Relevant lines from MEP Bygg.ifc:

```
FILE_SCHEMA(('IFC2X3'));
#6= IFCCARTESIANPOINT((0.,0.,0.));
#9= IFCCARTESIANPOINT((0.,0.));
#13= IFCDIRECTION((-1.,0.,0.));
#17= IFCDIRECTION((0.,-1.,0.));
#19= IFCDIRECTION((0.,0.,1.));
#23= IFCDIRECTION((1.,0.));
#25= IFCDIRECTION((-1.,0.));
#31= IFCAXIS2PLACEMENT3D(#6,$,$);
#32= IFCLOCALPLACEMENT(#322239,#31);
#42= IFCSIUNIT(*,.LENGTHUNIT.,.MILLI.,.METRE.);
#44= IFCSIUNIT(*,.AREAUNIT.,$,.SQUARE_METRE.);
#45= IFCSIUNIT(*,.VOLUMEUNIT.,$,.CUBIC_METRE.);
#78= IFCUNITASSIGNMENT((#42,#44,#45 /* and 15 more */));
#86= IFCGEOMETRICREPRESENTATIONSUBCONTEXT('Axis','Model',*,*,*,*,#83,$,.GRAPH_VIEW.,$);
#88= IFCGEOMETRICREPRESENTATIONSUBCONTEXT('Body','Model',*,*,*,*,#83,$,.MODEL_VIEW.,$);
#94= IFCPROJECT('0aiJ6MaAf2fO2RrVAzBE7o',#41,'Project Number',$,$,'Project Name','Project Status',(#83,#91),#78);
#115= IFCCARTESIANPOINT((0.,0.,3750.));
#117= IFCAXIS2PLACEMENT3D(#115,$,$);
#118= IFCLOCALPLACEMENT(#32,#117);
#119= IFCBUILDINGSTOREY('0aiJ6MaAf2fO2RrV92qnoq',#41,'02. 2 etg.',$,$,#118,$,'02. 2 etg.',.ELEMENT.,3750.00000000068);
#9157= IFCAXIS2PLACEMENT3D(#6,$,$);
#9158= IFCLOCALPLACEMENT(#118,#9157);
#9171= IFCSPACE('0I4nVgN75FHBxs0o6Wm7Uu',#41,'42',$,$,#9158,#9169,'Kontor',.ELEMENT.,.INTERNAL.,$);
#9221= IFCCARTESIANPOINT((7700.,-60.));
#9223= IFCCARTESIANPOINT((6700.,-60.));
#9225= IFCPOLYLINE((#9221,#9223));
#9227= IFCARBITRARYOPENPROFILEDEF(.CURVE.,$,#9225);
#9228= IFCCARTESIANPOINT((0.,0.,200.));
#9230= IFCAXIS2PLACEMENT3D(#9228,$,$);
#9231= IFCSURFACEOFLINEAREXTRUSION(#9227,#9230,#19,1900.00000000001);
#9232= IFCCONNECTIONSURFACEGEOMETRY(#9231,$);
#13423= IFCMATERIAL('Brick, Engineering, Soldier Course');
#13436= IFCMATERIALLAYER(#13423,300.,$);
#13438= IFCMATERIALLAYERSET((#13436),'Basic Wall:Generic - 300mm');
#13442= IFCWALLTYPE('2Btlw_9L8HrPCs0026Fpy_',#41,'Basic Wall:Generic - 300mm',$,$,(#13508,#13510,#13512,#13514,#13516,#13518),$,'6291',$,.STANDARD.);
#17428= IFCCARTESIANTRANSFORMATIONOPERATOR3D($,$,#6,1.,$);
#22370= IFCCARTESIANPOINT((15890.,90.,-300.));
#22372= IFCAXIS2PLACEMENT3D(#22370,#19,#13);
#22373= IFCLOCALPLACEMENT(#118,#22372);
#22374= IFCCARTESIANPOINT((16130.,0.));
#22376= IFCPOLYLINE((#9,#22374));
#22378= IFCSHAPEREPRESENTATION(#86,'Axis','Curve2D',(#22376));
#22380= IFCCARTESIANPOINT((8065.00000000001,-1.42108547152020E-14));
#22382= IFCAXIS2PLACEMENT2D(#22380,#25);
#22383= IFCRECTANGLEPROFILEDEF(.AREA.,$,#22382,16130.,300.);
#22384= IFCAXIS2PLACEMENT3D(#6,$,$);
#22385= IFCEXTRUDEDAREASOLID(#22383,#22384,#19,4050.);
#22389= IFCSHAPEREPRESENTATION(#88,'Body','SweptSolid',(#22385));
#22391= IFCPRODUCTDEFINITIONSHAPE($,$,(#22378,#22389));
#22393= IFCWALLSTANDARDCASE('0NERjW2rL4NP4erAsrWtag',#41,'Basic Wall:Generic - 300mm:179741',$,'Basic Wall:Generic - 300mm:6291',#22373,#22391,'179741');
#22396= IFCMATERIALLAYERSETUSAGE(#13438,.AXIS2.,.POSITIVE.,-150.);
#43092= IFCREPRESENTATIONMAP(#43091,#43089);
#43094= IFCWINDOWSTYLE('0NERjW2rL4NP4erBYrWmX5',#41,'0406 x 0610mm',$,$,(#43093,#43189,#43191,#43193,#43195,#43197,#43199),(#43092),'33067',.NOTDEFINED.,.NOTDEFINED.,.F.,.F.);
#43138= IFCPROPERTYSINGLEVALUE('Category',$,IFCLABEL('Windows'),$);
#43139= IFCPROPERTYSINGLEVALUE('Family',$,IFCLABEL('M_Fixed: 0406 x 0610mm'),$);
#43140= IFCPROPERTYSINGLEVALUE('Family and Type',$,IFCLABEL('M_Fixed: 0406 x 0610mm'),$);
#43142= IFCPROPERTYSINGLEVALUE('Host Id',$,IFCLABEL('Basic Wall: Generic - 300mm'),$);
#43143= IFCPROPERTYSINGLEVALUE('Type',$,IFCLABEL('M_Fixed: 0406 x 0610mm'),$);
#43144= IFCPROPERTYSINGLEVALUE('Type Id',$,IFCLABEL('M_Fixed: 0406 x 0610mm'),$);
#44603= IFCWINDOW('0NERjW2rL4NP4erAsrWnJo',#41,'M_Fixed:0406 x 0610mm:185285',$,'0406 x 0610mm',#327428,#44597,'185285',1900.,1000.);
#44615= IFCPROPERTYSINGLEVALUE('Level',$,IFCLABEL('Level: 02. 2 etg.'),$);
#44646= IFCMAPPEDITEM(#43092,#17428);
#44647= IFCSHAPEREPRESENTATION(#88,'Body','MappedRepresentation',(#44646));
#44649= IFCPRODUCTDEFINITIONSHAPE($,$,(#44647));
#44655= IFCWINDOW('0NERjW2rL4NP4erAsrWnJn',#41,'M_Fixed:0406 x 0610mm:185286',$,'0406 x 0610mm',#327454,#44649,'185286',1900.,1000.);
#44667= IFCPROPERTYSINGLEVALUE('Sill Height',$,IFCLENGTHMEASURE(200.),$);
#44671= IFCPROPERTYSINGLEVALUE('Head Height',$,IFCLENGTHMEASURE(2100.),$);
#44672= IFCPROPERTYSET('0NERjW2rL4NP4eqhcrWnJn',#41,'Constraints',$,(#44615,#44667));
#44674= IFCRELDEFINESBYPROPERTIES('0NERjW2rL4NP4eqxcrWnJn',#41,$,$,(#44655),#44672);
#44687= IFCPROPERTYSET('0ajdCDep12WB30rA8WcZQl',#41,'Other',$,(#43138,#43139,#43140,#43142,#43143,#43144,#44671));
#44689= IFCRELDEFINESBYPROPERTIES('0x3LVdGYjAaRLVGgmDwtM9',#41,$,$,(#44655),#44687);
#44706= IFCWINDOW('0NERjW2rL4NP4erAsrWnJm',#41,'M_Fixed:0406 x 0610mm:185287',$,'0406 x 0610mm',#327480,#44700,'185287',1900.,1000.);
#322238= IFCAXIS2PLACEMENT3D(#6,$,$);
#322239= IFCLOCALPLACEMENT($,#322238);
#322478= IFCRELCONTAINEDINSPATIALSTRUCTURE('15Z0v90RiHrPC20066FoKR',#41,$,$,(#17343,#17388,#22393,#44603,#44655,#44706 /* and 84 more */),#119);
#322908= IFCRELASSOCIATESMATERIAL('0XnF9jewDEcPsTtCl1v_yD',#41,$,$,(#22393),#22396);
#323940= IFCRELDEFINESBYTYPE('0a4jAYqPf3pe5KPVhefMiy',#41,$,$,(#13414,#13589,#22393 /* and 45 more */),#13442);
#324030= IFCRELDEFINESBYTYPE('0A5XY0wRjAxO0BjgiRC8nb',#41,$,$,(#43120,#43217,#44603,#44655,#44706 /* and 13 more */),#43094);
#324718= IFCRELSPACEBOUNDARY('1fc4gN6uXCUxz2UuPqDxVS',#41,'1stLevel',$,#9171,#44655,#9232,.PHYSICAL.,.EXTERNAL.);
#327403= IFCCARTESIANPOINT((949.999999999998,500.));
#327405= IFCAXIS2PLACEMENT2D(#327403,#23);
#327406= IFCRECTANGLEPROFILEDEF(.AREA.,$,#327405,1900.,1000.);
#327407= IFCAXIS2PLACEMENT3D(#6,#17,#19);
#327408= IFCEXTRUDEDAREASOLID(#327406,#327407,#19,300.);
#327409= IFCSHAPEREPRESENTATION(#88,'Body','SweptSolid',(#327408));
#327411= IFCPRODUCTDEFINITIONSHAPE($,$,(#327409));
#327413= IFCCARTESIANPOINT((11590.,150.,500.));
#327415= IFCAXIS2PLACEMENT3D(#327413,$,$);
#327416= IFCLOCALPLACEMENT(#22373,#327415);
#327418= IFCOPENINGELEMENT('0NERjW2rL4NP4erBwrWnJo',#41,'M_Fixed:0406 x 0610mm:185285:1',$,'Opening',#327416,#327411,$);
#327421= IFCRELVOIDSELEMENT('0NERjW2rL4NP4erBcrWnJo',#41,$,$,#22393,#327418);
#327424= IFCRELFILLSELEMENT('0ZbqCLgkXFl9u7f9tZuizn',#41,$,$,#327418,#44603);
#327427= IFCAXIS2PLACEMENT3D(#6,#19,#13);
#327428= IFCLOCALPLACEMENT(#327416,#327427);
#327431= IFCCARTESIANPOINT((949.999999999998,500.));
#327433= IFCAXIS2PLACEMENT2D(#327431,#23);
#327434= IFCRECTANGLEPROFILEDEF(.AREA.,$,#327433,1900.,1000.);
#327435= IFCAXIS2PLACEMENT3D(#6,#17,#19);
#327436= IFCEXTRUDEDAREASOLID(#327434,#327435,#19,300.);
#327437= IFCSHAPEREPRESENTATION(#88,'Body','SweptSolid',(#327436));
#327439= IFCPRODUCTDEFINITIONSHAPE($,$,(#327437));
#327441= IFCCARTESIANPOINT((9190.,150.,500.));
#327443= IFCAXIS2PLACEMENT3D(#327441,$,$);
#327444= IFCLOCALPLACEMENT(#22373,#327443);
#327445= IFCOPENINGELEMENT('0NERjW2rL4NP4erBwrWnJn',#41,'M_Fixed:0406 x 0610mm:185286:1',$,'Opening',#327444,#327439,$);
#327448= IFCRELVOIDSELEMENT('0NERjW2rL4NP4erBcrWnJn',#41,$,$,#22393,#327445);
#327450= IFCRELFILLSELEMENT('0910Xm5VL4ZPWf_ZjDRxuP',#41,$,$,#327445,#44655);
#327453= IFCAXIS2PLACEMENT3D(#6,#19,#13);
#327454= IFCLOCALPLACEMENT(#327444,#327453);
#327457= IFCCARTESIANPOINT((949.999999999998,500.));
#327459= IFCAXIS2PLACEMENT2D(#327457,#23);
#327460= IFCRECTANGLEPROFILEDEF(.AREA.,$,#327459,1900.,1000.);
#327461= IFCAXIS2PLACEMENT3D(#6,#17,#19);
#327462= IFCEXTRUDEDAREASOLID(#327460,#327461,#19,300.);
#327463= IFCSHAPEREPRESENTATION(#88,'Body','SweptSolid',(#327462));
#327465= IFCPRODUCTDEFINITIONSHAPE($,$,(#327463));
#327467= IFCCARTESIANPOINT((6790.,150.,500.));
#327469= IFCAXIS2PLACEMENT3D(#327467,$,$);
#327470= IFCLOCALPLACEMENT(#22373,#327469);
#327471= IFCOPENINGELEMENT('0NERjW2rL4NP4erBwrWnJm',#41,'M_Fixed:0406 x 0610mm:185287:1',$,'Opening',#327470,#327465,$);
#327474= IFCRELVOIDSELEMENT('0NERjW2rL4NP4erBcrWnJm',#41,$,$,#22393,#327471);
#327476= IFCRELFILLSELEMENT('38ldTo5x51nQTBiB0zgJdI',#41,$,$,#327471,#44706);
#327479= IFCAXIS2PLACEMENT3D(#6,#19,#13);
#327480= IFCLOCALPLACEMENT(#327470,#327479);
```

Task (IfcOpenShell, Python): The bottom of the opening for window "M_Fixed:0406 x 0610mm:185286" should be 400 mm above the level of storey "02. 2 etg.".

```python
import numpy as np
import ifcopenshell
import ifcopenshell.api.geometry
import ifcopenshell.api.pset
import ifcopenshell.geom
import ifcopenshell.util.element
import ifcopenshell.util.placement
import ifcopenshell.util.shape
import ifcopenshell.util.unit

model = ifcopenshell.open("MEP Bygg.ifc")
unit_scale = ifcopenshell.util.unit.calculate_unit_scale(model)

window = model.by_guid("0NERjW2rL4NP4erAsrWnJn")
opening = window.FillsVoids[0].RelatingOpeningElement
storey = ifcopenshell.util.element.get_container(window, ifc_class="IfcBuildingStorey")
level = ifcopenshell.util.placement.get_local_placement(storey.ObjectPlacement)[2, 3]

# The opening's origin need not be at the sill, so measure its lowest point.
shape = ifcopenshell.geom.create_shape(ifcopenshell.geom.settings(), opening)
bottom = ifcopenshell.util.shape.get_shape_bottom_elevation(shape, shape.geometry) / unit_scale
dz = level + 400.0 - bottom

shift = np.array([0.0, 0.0, dz])
# The window is placed relative to its opening, so it follows when the opening moves.
matrix = ifcopenshell.util.placement.get_local_placement(opening.ObjectPlacement)
matrix[:3, 3] += shift
ifcopenshell.api.geometry.edit_object_placement(
    model, product=opening, matrix=matrix, is_si=False, should_transform_children=True
)

# Space boundary surfaces are stored in each space's coordinates; move them too.
for rel in window.ProvidesBoundaries:
    if not rel.ConnectionGeometry:
        continue
    surface = rel.ConnectionGeometry.SurfaceOnRelatingElement
    space_matrix = ifcopenshell.util.placement.get_local_placement(rel.RelatingSpace.ObjectPlacement)
    point = np.array(surface.Position.Location.Coordinates) + space_matrix[:3, :3].T @ shift
    surface.Position = model.createIfcAxis2Placement3D(
        model.createIfcCartesianPoint(point.tolist()), surface.Position.Axis, surface.Position.RefDirection
    )

# Keep the stored heights in step.
pset = model.by_id(ifcopenshell.util.element.get_pset(window, "Constraints", should_inherit=False)["id"])
ifcopenshell.api.pset.edit_pset(model, pset=pset, properties={
    "Sill Height": model.create_entity("IfcLengthMeasure", ifcopenshell.util.element.get_pset(window, "Constraints", "Sill Height") + dz),
})
pset = model.by_id(ifcopenshell.util.element.get_pset(window, "Other", should_inherit=False)["id"])
ifcopenshell.api.pset.edit_pset(model, pset=pset, properties={
    "Head Height": model.create_entity("IfcLengthMeasure", ifcopenshell.util.element.get_pset(window, "Other", "Head Height") + dz),
})

print(f"moved by {dz * unit_scale:+.3f} m")

model.write("MEP Bygg_edited.ifc")
```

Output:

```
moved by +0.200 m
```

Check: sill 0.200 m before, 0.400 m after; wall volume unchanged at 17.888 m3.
